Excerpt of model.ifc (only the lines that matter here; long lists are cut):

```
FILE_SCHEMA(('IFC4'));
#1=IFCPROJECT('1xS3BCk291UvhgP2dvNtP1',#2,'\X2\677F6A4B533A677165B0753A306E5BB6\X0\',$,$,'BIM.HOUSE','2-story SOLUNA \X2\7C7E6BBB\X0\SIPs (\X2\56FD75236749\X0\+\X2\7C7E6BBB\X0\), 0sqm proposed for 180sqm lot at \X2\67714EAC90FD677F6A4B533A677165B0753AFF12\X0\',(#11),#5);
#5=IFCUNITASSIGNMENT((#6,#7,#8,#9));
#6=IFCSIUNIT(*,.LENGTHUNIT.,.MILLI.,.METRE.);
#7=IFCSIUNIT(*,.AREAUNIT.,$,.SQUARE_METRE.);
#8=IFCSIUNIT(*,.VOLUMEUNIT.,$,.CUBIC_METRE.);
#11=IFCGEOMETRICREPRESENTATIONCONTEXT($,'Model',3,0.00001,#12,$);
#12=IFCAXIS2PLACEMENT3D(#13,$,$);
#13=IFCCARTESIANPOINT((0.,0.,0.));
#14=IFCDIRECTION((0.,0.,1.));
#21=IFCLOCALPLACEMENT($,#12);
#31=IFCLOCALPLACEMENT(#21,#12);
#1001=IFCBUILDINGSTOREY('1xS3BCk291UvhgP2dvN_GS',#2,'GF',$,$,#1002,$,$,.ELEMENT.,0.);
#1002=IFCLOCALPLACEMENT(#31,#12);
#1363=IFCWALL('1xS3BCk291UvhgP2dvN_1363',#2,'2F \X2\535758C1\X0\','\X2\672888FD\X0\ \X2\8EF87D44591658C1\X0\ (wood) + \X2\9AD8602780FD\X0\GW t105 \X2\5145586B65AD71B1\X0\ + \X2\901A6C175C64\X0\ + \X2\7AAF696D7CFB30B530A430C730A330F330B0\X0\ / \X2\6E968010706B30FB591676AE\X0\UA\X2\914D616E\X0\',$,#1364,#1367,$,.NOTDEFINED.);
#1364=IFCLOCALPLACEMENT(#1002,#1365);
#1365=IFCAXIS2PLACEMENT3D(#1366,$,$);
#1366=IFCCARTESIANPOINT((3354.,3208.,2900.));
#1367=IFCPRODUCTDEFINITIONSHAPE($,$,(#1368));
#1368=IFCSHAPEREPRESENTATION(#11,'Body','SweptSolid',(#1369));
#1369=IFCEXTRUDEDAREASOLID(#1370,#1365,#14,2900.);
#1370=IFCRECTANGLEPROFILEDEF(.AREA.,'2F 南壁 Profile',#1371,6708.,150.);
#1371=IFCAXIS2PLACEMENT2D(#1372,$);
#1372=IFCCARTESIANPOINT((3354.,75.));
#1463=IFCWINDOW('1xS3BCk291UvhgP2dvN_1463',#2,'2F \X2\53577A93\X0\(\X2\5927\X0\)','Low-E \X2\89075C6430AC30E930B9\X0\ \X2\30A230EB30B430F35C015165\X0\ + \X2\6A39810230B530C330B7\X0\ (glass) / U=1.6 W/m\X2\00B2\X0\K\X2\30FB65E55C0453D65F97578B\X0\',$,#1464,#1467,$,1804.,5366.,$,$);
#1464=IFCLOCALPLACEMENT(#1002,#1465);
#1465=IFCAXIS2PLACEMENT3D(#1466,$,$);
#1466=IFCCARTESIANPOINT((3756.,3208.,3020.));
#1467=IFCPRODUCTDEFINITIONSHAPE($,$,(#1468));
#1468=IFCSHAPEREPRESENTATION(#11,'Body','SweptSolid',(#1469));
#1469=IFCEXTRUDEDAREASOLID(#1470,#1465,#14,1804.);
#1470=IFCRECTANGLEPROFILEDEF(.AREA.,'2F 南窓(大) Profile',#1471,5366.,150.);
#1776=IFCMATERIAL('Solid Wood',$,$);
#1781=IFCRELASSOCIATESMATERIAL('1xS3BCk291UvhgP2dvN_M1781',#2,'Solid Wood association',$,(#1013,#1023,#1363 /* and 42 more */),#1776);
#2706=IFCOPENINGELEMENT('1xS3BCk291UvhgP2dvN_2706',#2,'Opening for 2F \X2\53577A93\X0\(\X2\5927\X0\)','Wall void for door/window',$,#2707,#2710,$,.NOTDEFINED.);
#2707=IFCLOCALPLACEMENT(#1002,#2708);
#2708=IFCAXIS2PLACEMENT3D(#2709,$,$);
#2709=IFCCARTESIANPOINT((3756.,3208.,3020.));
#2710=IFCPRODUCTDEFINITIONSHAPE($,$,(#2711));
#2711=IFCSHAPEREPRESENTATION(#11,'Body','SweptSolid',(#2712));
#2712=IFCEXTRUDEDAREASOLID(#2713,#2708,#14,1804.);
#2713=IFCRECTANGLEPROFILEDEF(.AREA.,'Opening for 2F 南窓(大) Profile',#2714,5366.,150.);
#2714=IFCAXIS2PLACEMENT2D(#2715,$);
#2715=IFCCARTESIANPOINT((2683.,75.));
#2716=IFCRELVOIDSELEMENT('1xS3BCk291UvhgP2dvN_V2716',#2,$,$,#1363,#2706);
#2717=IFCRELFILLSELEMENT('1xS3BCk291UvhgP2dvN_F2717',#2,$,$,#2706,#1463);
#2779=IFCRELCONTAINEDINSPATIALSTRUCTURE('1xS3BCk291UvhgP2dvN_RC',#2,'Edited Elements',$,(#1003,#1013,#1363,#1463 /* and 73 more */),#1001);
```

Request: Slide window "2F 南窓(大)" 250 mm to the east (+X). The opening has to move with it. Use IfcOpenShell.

```python
import ifcopenshell
import ifcopenshell.api.geometry
import ifcopenshell.util.placement
import ifcopenshell.util.unit

model = ifcopenshell.open("model.ifc")
unit_scale = ifcopenshell.util.unit.calculate_unit_scale(model)

window = model.by_guid("1xS3BCk291UvhgP2dvN_1463")
opening = window.FillsVoids[0].RelatingOpeningElement
wall = opening.VoidsElements[0].RelatingBuildingElement

wall_matrix = ifcopenshell.util.placement.get_local_placement(wall.ObjectPlacement)
shift = wall_matrix[:3, 0] * 0.25 / unit_scale
before = ifcopenshell.util.placement.get_local_placement(window.ObjectPlacement)[:3, 3].copy()

# The window is not placed relative to its opening, so move both.
for product in (opening, window):
    matrix = ifcopenshell.util.placement.get_local_placement(product.ObjectPlacement)
    matrix[:3, 3] += shift
    ifcopenshell.api.geometry.edit_object_placement(model, product=product, matrix=matrix, is_si=False)

after = ifcopenshell.util.placement.get_local_placement(window.ObjectPlacement)[:3, 3]
print("window moved by", (after - before).round(3) + 0.0)

model.write("model-out.ifc")
```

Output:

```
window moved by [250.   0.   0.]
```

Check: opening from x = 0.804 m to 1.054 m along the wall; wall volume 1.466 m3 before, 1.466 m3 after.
